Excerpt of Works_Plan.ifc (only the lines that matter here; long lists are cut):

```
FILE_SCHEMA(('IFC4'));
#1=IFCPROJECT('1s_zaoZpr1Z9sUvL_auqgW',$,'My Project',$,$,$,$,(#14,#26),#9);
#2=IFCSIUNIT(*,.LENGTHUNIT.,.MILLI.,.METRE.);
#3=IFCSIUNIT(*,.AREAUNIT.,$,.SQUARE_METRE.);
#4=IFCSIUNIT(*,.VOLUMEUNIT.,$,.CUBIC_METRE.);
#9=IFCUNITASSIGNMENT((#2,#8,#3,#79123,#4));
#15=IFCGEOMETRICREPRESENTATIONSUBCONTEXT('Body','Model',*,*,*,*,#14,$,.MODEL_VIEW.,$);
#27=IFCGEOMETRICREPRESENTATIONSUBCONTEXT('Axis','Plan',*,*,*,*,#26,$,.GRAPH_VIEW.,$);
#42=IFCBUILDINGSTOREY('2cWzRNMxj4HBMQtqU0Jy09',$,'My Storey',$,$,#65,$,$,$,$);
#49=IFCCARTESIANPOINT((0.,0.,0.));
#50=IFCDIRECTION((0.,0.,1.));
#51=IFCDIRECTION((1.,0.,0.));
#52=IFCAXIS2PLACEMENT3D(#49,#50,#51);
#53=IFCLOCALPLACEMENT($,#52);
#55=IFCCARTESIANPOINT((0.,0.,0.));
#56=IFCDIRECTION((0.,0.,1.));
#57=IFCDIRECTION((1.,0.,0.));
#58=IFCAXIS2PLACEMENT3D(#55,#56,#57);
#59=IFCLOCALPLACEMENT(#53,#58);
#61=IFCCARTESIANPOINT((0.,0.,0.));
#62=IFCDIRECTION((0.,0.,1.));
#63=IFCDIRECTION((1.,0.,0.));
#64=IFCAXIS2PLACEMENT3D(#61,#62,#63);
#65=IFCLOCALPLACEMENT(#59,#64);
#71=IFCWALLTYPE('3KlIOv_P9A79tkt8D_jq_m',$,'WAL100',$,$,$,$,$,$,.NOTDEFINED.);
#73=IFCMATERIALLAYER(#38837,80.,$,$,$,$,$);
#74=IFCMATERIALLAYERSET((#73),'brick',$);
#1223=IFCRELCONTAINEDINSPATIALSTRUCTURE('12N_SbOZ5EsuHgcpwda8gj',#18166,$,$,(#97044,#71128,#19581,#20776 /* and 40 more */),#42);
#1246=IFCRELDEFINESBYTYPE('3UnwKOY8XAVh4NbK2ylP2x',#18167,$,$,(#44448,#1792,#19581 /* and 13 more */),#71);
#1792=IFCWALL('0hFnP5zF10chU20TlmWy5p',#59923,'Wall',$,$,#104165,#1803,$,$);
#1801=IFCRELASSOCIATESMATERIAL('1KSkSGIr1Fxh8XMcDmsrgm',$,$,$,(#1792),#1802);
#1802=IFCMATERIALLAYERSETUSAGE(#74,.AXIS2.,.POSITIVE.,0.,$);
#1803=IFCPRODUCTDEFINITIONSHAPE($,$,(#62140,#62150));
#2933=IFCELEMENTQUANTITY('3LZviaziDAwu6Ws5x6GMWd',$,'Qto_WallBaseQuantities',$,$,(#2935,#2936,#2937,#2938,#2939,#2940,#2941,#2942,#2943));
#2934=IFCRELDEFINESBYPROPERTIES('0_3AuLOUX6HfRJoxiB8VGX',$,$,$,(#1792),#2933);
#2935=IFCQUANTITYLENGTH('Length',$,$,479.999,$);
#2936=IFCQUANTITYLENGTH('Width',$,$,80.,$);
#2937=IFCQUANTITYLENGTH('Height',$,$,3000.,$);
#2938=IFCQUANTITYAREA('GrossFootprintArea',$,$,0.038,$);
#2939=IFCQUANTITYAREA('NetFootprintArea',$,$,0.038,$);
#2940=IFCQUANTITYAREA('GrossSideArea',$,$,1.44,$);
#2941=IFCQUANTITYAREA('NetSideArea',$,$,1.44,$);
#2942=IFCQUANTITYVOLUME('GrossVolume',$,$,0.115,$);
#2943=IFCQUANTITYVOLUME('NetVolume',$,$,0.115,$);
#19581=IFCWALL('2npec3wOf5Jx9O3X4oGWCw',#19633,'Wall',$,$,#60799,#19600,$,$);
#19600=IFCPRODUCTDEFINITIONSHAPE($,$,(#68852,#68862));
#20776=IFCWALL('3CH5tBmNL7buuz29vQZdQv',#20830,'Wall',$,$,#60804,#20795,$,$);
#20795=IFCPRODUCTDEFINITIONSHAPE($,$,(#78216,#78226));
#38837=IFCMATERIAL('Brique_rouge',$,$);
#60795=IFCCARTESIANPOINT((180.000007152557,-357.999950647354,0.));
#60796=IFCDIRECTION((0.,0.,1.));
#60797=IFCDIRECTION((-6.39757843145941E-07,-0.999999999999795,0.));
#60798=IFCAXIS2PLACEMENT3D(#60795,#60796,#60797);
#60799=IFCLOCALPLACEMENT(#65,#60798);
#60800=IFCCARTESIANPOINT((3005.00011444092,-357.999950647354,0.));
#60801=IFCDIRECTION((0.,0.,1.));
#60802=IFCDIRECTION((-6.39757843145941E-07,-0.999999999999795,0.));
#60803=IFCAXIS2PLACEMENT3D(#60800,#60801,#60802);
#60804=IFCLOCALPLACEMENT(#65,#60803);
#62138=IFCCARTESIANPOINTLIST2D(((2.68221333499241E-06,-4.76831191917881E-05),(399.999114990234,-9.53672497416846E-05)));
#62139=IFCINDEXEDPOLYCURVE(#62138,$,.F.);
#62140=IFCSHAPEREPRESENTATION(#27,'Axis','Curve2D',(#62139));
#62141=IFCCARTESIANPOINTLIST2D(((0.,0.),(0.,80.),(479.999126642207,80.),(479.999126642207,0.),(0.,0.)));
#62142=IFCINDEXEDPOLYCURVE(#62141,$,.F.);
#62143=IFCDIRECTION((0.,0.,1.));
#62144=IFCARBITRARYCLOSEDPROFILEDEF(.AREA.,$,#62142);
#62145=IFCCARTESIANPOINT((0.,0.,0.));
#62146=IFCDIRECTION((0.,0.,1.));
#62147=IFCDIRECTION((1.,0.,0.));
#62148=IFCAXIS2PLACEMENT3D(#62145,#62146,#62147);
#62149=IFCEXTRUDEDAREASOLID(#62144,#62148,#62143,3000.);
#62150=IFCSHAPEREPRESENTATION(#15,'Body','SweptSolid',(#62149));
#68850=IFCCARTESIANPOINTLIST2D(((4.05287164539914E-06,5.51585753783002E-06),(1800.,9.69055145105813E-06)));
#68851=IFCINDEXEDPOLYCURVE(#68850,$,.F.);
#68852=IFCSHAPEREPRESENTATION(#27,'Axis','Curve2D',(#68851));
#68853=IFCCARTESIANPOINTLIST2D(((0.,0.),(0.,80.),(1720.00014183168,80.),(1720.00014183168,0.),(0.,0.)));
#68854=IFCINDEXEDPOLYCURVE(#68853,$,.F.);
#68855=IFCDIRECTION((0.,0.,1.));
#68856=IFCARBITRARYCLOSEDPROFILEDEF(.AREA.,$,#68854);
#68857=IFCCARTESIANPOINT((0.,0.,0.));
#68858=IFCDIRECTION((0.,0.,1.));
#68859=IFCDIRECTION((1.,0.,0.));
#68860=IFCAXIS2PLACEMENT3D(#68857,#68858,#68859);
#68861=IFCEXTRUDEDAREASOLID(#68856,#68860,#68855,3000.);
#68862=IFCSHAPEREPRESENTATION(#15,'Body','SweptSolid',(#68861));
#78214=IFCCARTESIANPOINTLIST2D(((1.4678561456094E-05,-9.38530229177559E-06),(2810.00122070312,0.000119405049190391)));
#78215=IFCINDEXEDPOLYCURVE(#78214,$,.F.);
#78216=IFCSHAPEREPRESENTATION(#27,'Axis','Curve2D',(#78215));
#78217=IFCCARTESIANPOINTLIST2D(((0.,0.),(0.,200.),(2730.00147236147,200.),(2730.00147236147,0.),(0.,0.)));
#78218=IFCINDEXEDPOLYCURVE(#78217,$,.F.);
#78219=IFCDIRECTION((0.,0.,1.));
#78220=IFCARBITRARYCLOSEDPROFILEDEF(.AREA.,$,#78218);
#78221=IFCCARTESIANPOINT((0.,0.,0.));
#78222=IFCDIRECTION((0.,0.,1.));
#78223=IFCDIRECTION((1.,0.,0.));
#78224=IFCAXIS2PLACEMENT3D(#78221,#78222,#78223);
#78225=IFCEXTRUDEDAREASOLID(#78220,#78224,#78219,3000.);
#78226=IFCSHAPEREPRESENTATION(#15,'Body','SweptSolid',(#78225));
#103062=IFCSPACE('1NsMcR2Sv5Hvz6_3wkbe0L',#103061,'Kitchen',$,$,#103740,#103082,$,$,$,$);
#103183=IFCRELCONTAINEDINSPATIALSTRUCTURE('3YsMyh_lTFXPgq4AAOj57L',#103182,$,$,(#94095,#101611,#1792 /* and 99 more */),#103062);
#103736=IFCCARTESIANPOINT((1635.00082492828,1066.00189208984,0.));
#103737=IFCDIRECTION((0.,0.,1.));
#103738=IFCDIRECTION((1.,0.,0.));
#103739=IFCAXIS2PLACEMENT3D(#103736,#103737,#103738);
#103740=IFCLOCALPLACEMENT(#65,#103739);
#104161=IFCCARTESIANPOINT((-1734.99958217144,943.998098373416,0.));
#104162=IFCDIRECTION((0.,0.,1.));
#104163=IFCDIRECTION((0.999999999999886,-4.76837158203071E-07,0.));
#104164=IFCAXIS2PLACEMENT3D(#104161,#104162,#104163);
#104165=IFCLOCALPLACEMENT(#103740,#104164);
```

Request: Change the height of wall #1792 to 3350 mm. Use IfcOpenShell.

```python
import ifcopenshell
import ifcopenshell.api.pset
import ifcopenshell.geom
import ifcopenshell.util.element
import ifcopenshell.util.representation
import ifcopenshell.util.shape
import ifcopenshell.util.unit

model = ifcopenshell.open("Works_Plan.ifc")
unit_scale = ifcopenshell.util.unit.calculate_unit_scale(model)
area_scale = ifcopenshell.util.unit.calculate_unit_scale(model, "AREAUNIT")
volume_scale = ifcopenshell.util.unit.calculate_unit_scale(model, "VOLUMEUNIT")
settings = ifcopenshell.geom.settings()


def volume(element):
    """Net volume in cubic metres, openings subtracted."""
    shape = ifcopenshell.geom.create_shape(settings, element)
    return ifcopenshell.util.shape.get_volume(shape.geometry)


wall = model.by_guid("0hFnP5zF10chU20TlmWy5p")
before = volume(wall)

body = ifcopenshell.util.representation.get_representation(wall, "Model", "Body")
solid = body.Items[0]
old_height = solid.Depth
solid.Depth = 3.35 / unit_scale
after = volume(wall)
thickness = 0.08  # wall thickness in metres

# Update the stored height, areas and volumes.
qto = model.by_id(ifcopenshell.util.element.get_pset(wall, "Qto_WallBaseQuantities", should_inherit=False)["id"])
ifcopenshell.api.pset.edit_qto(model, qto=qto, properties={
    "Height": solid.Depth,
    "GrossSideArea": ifcopenshell.util.element.get_pset(wall, "Qto_WallBaseQuantities", "GrossSideArea") * solid.Depth / old_height,
    "NetSideArea": after / thickness / area_scale,
    "GrossVolume": ifcopenshell.util.element.get_pset(wall, "Qto_WallBaseQuantities", "GrossVolume") * solid.Depth / old_height,
    "NetVolume": after / volume_scale,
})

print(f"height {old_height:g} -> {solid.Depth:g}, volume {before:.3f} -> {after:.3f} m3")

model.write("Works_Plan-out.ifc")
```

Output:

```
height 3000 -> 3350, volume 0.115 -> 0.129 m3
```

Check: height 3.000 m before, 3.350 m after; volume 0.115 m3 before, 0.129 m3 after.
